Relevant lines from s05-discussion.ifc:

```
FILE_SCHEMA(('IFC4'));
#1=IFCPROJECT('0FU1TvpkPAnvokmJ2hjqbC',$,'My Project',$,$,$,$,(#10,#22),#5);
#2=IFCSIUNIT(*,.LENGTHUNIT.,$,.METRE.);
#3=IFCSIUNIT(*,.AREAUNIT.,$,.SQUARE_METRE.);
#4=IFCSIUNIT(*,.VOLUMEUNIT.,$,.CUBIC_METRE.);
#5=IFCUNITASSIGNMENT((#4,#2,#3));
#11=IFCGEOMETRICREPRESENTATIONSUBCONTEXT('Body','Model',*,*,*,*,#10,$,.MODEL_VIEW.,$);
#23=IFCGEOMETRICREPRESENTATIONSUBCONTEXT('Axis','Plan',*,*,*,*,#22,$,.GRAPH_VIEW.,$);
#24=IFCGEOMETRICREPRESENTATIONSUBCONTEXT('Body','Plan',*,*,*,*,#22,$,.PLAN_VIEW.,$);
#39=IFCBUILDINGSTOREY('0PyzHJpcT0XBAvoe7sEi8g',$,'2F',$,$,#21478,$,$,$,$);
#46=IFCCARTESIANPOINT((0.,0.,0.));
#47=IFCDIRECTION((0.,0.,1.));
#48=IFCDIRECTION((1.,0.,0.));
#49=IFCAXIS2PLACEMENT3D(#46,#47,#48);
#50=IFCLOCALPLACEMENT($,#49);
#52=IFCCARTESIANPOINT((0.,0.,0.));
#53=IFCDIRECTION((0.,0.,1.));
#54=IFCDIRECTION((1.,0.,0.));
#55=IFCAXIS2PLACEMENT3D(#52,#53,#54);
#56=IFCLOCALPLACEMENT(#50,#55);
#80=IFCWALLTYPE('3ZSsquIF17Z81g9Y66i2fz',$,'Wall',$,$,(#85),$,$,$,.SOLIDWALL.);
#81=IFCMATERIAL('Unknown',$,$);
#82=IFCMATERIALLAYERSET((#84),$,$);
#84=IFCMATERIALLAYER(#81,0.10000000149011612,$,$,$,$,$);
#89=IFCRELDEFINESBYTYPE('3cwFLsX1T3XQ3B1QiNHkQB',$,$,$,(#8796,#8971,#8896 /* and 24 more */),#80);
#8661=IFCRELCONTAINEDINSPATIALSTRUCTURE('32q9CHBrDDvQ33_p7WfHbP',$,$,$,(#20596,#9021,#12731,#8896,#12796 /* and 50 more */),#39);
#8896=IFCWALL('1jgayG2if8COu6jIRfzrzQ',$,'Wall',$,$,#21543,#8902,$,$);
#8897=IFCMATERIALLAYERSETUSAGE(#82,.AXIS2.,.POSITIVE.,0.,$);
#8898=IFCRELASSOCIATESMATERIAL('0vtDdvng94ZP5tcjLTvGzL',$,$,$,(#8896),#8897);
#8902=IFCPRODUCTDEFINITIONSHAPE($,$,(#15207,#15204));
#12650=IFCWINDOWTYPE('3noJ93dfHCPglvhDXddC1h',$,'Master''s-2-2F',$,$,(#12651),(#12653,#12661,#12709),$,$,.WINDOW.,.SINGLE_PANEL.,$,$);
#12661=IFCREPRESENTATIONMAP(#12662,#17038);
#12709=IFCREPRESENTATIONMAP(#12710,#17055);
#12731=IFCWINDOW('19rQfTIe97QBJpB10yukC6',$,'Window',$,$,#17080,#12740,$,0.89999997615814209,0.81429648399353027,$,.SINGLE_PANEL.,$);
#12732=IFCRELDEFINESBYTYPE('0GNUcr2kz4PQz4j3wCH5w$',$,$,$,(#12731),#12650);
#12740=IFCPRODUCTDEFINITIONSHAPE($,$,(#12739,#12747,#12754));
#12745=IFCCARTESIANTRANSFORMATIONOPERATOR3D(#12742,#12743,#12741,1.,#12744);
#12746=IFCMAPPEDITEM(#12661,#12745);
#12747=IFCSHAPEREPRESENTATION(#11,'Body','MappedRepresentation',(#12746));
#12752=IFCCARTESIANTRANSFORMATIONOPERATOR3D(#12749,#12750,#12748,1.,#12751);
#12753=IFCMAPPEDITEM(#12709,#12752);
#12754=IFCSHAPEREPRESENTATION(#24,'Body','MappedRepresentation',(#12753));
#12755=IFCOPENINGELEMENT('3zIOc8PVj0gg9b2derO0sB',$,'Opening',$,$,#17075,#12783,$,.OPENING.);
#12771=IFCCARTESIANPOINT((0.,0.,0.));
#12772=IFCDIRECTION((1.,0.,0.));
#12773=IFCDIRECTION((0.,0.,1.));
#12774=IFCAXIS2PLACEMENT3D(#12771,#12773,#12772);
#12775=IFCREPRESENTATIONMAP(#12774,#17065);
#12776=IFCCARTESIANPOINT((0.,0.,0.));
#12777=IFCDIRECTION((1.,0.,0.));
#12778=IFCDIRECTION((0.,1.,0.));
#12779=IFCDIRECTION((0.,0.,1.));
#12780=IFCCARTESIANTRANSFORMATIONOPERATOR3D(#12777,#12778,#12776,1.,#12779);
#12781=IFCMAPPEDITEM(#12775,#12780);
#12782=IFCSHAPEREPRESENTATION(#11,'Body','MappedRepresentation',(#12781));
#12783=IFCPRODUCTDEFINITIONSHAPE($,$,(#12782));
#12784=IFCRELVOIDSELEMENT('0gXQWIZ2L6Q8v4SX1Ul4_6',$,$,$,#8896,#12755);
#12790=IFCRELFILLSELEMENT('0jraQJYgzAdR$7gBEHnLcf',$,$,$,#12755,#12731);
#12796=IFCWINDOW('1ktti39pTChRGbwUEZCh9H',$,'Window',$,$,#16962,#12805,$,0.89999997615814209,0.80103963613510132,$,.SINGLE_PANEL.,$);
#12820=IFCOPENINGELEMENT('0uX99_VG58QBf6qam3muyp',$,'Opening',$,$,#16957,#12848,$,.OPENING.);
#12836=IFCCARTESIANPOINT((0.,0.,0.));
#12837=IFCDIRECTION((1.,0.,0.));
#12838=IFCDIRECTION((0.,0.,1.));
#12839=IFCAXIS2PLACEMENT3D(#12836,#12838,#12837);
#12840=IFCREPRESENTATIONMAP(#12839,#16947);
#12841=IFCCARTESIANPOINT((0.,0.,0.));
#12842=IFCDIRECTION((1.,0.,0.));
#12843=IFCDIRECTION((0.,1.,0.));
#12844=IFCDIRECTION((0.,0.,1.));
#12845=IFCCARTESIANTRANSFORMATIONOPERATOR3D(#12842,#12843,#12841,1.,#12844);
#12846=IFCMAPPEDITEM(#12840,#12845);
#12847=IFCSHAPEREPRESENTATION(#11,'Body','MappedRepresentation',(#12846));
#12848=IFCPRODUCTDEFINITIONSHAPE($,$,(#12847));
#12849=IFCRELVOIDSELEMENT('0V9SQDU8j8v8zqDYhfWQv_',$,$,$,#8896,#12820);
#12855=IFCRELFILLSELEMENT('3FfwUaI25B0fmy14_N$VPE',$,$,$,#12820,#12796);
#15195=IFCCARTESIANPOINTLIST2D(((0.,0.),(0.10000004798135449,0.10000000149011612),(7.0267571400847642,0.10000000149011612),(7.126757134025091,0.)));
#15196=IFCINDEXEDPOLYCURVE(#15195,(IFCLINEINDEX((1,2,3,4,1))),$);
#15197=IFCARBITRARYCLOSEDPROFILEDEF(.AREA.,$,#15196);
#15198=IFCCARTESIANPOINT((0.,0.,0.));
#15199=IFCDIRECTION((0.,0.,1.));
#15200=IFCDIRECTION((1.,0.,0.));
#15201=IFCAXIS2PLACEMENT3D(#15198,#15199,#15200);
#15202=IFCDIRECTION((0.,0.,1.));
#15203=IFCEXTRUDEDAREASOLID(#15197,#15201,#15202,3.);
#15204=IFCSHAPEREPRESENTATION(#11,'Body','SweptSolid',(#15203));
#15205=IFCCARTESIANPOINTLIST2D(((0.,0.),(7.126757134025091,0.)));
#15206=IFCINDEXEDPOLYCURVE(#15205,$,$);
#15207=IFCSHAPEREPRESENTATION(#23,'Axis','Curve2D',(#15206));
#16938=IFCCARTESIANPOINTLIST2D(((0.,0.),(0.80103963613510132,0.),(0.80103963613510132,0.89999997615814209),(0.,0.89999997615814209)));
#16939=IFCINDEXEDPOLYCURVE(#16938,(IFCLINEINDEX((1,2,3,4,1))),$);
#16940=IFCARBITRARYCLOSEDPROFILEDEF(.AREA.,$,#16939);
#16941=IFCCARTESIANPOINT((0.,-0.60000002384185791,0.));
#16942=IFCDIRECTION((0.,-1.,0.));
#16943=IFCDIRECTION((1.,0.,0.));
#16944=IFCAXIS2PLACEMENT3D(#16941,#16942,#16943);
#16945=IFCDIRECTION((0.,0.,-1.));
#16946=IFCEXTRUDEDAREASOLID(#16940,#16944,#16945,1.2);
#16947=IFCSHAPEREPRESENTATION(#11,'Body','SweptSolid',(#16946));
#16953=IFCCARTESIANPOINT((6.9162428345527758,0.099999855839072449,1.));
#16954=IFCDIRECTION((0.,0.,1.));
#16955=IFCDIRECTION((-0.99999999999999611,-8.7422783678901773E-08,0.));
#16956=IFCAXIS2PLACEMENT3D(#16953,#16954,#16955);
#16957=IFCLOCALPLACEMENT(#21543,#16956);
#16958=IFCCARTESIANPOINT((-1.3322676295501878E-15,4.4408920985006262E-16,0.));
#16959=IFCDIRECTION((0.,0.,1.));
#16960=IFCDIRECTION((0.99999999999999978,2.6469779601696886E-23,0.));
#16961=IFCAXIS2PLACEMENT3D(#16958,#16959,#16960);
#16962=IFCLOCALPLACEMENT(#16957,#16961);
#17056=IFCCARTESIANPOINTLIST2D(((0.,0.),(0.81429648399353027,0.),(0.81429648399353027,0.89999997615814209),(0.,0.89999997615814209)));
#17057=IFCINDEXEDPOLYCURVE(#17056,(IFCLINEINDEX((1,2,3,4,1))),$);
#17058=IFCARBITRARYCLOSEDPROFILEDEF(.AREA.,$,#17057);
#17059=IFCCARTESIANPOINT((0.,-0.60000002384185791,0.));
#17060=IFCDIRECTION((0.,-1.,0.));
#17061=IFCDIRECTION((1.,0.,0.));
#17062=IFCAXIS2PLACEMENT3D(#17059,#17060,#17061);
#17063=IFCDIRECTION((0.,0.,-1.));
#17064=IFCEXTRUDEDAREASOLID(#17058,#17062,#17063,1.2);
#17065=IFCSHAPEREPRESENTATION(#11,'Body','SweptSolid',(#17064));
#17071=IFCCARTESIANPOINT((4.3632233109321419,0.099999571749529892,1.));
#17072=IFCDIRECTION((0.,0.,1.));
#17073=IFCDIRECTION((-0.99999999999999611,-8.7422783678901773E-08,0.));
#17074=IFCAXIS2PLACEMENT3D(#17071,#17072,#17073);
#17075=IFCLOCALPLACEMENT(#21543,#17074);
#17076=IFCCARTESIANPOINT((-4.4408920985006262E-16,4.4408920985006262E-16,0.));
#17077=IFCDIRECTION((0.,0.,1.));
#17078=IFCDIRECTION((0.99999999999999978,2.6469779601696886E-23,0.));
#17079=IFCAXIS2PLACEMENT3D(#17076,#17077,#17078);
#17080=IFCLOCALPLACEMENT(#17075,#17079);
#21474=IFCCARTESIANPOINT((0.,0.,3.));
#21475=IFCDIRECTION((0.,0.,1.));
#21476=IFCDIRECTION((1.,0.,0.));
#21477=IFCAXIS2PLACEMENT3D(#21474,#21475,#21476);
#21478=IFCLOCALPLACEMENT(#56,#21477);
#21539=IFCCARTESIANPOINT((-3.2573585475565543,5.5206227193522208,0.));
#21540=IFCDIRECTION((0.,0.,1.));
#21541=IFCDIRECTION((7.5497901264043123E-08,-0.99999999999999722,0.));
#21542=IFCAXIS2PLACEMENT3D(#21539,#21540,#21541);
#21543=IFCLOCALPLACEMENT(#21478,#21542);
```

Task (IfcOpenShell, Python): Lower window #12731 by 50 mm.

```python
import numpy as np
import ifcopenshell
import ifcopenshell.api.geometry
import ifcopenshell.util.placement
import ifcopenshell.util.unit

model = ifcopenshell.open("s05-discussion.ifc")
unit_scale = ifcopenshell.util.unit.calculate_unit_scale(model)

window = model.by_guid("19rQfTIe97QBJpB10yukC6")
opening = window.FillsVoids[0].RelatingOpeningElement
dz = -0.05 / unit_scale

shift = np.array([0.0, 0.0, dz])
# The window is placed relative to its opening, so it follows when the opening moves.
matrix = ifcopenshell.util.placement.get_local_placement(opening.ObjectPlacement)
matrix[:3, 3] += shift
ifcopenshell.api.geometry.edit_object_placement(
    model, product=opening, matrix=matrix, is_si=False, should_transform_children=True
)

print(f"moved by {dz * unit_scale:+.3f} m")

model.write("s05-discussion_rev.ifc")
```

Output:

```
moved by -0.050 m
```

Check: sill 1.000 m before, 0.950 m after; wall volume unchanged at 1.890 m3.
